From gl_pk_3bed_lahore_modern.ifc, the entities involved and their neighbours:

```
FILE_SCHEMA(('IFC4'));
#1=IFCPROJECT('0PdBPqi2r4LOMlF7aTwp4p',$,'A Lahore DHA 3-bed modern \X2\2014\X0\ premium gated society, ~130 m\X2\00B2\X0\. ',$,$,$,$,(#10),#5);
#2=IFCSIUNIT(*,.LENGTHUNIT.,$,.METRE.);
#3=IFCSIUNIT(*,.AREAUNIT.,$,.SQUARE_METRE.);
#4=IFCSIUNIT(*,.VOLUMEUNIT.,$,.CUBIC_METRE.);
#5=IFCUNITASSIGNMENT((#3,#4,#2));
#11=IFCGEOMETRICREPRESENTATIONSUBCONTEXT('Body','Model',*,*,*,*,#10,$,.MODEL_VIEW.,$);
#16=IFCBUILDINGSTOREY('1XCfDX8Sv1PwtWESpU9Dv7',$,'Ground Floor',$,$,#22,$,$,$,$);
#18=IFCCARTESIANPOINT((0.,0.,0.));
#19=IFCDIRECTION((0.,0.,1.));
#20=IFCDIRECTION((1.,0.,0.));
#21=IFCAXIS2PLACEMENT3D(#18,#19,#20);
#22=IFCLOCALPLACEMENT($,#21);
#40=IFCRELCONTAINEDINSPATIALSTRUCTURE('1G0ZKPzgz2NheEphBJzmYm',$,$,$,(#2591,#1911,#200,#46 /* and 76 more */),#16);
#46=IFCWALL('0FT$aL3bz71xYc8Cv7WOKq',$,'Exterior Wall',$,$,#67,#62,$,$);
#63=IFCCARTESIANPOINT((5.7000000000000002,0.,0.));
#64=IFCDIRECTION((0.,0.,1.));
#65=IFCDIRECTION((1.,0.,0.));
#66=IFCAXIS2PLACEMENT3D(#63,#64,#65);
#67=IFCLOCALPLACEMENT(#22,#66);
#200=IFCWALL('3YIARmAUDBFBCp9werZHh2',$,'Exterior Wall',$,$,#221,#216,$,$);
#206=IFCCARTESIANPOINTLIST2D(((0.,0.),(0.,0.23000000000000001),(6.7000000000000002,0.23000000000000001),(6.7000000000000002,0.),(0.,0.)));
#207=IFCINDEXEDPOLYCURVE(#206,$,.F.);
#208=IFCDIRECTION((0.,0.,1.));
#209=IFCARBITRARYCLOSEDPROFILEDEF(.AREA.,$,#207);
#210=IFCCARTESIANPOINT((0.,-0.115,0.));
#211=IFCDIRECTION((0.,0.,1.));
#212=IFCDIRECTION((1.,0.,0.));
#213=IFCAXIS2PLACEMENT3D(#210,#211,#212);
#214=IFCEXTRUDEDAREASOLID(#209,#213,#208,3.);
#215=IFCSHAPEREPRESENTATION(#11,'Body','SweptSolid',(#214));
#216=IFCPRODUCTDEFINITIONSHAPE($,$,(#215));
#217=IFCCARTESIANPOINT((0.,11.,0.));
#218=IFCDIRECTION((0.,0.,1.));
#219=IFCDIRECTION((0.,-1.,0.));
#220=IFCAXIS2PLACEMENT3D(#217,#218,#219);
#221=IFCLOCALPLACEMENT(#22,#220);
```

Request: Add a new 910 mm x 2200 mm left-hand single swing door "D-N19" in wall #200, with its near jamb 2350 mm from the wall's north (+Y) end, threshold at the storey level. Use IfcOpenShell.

```python
import numpy as np
import ifcopenshell
import ifcopenshell.api.feature
import ifcopenshell.api.geometry
import ifcopenshell.api.root
import ifcopenshell.api.spatial
import ifcopenshell.geom
import ifcopenshell.util.element
import ifcopenshell.util.placement
import ifcopenshell.util.representation
import ifcopenshell.util.shape
import ifcopenshell.util.unit

model = ifcopenshell.open("gl_pk_3bed_lahore_modern.ifc")
unit_scale = ifcopenshell.util.unit.calculate_unit_scale(model)
settings = ifcopenshell.geom.settings()


def volume(element):
    """Net volume in cubic metres, openings subtracted."""
    shape = ifcopenshell.geom.create_shape(settings, element)
    return ifcopenshell.util.shape.get_volume(shape.geometry)


wall = model.by_guid("3YIARmAUDBFBCp9werZHh2")
storey = ifcopenshell.util.element.get_container(wall, ifc_class="IfcBuildingStorey")
context = ifcopenshell.util.representation.get_context(model, "Model", "Body", "MODEL_VIEW")
before = volume(wall)

width, height, from_end, sill = 0.91, 2.2, 2.35, 0.0  # metres

# The wall runs along its own X axis, and the end named is its -X end.
wall_shape = ifcopenshell.geom.create_shape(settings, wall)
x, y, z = ifcopenshell.util.shape.get_vertices(wall_shape.geometry).T
start = x.min() + from_end
face, thickness = float(y.min()), float(y.max() - y.min())
wall_matrix = ifcopenshell.util.placement.get_local_placement(wall.ObjectPlacement)
level = ifcopenshell.util.placement.get_local_placement(storey.ObjectPlacement)[2, 3]


def in_wall(x, y):
    """Placement at x, y metres in the wall's axes, at sill height."""
    matrix = wall_matrix.copy()
    matrix[:, 3] = wall_matrix @ np.array([x / unit_scale, y / unit_scale, 0.0, 1.0])
    matrix[2, 3] = level + sill / unit_scale
    return matrix


# Opening: a box that overshoots both wall faces by 50 mm.
opening = ifcopenshell.api.root.create_entity(model, ifc_class="IfcOpeningElement", predefined_type="OPENING")
box = ifcopenshell.api.geometry.add_wall_representation(
    model, context=context, length=width, height=height, thickness=thickness + 0.1
)
ifcopenshell.api.geometry.assign_representation(model, product=opening, representation=box)
ifcopenshell.api.geometry.edit_object_placement(model, product=opening, matrix=in_wall(start, face - 0.05), is_si=False)
ifcopenshell.api.feature.add_feature(model, feature=opening, element=wall)

door = ifcopenshell.api.root.create_entity(model, ifc_class="IfcDoor", name="D-N19", predefined_type="DOOR")
door.OverallWidth, door.OverallHeight = width / unit_scale, height / unit_scale
door.OperationType = "SINGLE_SWING_LEFT"
body = ifcopenshell.api.geometry.add_door_representation(
    model,
    context=context,
    overall_width=door.OverallWidth,
    overall_height=door.OverallHeight,
    operation_type="SINGLE_SWING_LEFT",
    lining_properties={"LiningDepth": thickness / unit_scale, "ThresholdDepth": thickness / unit_scale},
)
ifcopenshell.api.geometry.assign_representation(model, product=door, representation=body)
ifcopenshell.api.spatial.assign_container(model, products=[door], relating_structure=storey)
ifcopenshell.api.feature.add_filling(model, opening=opening, element=door)

# The lining spans the wall, so the door starts at the wall face.
ifcopenshell.api.geometry.edit_object_placement(model, product=door, matrix=in_wall(start, face), is_si=False)

after = volume(wall)

print(f"wall volume {before:.3f} -> {after:.3f} m3")

model.write("gl_pk_3bed_lahore_modern_rev.ifc")
```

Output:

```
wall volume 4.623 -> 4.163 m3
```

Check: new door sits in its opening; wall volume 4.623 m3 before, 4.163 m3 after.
